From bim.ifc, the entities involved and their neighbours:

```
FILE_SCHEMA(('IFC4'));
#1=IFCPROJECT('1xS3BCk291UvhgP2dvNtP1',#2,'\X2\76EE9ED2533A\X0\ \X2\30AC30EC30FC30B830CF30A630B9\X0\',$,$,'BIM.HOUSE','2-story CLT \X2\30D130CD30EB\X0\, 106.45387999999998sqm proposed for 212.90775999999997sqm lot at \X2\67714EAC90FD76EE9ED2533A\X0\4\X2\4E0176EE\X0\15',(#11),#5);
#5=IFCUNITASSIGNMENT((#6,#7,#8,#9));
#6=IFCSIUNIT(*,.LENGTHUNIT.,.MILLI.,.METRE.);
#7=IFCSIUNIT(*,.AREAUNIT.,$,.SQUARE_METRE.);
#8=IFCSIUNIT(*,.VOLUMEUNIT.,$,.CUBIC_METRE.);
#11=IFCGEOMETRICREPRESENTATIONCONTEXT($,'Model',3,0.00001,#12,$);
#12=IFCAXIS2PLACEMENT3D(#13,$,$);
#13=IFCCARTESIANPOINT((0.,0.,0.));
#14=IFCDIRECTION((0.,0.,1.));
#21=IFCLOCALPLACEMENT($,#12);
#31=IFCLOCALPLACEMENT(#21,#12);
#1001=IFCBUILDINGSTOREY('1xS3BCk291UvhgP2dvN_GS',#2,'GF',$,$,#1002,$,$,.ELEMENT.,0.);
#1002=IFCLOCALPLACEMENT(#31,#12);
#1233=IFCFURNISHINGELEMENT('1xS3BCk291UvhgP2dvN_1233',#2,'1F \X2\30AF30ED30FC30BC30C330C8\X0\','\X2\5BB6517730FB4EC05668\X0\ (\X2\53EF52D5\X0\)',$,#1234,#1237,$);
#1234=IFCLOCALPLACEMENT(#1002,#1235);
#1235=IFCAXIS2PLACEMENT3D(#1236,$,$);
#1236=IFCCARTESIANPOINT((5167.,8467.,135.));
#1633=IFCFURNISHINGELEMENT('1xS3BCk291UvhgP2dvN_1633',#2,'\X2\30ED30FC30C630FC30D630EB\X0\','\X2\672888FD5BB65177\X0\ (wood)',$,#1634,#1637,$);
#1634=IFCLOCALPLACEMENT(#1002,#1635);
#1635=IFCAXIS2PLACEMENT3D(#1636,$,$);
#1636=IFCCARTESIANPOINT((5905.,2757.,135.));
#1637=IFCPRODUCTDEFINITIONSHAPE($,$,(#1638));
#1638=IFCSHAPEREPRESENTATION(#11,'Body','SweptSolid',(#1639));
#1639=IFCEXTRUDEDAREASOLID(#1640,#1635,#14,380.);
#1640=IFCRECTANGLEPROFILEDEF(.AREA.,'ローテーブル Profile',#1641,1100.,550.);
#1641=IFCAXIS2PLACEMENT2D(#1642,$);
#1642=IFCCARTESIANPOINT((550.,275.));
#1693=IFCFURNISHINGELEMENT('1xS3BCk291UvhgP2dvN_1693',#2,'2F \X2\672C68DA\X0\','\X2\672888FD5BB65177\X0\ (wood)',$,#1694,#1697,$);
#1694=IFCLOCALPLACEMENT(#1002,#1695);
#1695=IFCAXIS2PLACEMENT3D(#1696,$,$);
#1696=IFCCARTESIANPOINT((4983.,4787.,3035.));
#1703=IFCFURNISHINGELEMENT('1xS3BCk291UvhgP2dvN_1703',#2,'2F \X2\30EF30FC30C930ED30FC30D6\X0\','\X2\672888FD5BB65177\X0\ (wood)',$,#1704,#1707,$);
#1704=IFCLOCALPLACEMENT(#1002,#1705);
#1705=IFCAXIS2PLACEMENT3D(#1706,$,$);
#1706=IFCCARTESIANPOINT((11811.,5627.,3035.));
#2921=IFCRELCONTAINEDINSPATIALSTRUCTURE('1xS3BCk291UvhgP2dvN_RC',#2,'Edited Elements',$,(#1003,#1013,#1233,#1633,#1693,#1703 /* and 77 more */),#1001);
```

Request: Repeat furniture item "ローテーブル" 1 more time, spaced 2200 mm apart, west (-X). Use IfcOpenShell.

```python
import numpy as np
import ifcopenshell
import ifcopenshell.api.geometry
import ifcopenshell.api.root
import ifcopenshell.util.element
import ifcopenshell.util.placement
import ifcopenshell.util.unit

model = ifcopenshell.open("bim.ifc")
unit_scale = ifcopenshell.util.unit.calculate_unit_scale(model)


def reuse_history(source, copy):
    """copy_class also copies each property set's owner history, people and application; keep the originals."""
    for rel in copy.IsDefinedBy:
        if rel.is_a("IfcRelDefinesByProperties") and (history := rel.RelatingPropertyDefinition.OwnerHistory):
            rel.RelatingPropertyDefinition.OwnerHistory = source.OwnerHistory
            ifcopenshell.util.element.remove_deep2(model, history)


source = model.by_guid("1xS3BCk291UvhgP2dvN_1633")
base = ifcopenshell.util.placement.get_local_placement(source.ObjectPlacement)
step = np.array([-1.0, 0.0, 0.0]) * 2.2 / unit_scale

for i in range(1, 2):
    copy = ifcopenshell.api.root.copy_class(model, product=source)
    copy.Representation = ifcopenshell.util.element.copy_deep(
        model, source.Representation, exclude=["IfcGeometricRepresentationContext", "IfcRepresentationMap"]
    )
    reuse_history(source, copy)
    matrix = base.copy()
    matrix[:3, 3] += i * step
    print("added at", matrix[:3, 3].round(3) + 0.0)
    ifcopenshell.api.geometry.edit_object_placement(model, product=copy, matrix=matrix, is_si=False)

model.write("bim_updated.ifc")
```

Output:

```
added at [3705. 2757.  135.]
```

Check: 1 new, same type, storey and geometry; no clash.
